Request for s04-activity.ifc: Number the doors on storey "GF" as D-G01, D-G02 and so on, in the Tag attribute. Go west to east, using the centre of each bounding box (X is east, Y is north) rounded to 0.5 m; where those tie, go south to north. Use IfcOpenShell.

First a look at what the model holds.

```python
import ifcopenshell
import ifcopenshell.util.element
import ifcopenshell.util.placement

model = ifcopenshell.open("s04-activity.ifc")
print(model.schema)
storey = next(s for s in model.by_type("IfcBuildingStorey") if s.Name == "GF")
doors = [e for e in ifcopenshell.util.element.get_decomposition(storey) if e.is_a("IfcDoor")]
for e in sorted(doors, key=lambda e: e.id()):
    origin = ifcopenshell.util.placement.get_local_placement(e.ObjectPlacement)[:3, 3]
    print(e.id(), e.Tag, e.Name, origin.round(2) + 0.0, sep=" | ")
```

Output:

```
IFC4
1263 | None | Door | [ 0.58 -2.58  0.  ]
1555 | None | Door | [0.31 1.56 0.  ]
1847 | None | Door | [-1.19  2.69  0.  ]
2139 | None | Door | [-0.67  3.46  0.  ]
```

```python
import ifcopenshell
import ifcopenshell.geom
import ifcopenshell.util.element
import ifcopenshell.util.shape

model = ifcopenshell.open("s04-activity.ifc")
settings = ifcopenshell.geom.settings()
settings.set("use-world-coords", True)


def centre(element):
    shape = ifcopenshell.geom.create_shape(settings, element)
    return ifcopenshell.util.shape.get_bbox_centroid(shape.geometry)


storey = next(s for s in model.by_type("IfcBuildingStorey") if s.Name == "GF")
doors = [e for e in ifcopenshell.util.element.get_decomposition(storey) if e.is_a("IfcDoor")]

# Insertion points can sit at a corner or the storey origin, so sort by the geometry (in metres).
centres = {e: centre(e) for e in doors}
doors.sort(key=lambda e: (round(centres[e][0] / 0.5), centres[e][1]))

for i, e in enumerate(doors, start=1):
    number = f"D-G{i:02d}"
    e.Tag = number
    print(e.id(), number)

model.write("s04-activity_rev.ifc")
```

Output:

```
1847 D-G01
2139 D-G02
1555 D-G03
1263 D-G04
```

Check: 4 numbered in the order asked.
